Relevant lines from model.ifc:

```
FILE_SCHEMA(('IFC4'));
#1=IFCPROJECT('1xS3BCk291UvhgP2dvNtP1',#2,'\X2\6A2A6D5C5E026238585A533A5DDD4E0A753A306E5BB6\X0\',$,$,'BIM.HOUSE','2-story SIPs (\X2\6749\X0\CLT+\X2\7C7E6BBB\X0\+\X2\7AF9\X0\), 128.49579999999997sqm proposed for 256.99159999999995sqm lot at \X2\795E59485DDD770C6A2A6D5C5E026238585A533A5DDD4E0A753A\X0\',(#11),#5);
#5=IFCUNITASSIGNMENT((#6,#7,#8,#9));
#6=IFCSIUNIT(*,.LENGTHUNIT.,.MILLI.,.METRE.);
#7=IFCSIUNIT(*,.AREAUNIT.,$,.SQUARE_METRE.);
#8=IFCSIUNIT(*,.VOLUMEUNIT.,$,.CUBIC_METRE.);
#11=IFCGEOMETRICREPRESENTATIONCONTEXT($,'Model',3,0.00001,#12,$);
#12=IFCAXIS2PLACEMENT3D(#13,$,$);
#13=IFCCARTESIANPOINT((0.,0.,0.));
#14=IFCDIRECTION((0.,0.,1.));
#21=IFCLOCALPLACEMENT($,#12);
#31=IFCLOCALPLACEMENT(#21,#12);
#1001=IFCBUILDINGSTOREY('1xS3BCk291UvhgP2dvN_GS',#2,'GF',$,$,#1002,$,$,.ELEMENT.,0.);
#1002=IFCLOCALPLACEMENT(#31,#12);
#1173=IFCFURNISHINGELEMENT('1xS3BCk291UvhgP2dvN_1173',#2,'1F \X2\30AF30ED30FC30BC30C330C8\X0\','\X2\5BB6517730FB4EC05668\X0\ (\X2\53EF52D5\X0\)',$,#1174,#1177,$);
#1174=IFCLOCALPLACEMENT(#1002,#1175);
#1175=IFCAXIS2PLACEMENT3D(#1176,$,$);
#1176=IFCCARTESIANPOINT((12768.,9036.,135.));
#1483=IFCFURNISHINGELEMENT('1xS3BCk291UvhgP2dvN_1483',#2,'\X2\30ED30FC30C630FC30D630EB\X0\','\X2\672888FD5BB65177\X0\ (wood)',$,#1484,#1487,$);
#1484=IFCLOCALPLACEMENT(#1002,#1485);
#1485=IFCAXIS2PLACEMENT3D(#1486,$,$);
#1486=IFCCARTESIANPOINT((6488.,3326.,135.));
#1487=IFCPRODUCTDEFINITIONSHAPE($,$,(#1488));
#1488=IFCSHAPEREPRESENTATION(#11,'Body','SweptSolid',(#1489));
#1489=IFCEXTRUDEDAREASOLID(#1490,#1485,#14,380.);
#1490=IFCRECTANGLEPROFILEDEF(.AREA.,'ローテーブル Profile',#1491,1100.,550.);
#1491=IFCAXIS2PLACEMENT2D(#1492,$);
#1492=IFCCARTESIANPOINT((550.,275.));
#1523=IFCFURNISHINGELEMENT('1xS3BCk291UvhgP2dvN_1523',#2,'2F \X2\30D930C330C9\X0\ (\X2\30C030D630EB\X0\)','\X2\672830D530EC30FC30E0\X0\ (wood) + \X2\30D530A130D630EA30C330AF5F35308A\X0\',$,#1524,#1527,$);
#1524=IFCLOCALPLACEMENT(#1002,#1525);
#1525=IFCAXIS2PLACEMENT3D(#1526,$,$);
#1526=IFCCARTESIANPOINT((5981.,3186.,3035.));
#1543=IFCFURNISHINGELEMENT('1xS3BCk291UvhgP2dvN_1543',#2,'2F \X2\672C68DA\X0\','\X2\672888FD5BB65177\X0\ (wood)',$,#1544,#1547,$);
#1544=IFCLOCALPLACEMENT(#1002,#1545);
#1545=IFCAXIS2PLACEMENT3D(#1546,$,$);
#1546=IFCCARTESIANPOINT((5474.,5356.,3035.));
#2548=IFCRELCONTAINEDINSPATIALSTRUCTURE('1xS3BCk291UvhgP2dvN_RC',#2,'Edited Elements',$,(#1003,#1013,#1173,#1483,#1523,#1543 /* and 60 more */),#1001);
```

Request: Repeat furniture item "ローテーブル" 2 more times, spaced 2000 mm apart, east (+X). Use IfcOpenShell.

```python
import numpy as np
import ifcopenshell
import ifcopenshell.api.geometry
import ifcopenshell.api.root
import ifcopenshell.util.element
import ifcopenshell.util.placement
import ifcopenshell.util.unit

model = ifcopenshell.open("model.ifc")
unit_scale = ifcopenshell.util.unit.calculate_unit_scale(model)


def reuse_history(source, copy):
    """copy_class also copies each property set's owner history, people and application; keep the originals."""
    for rel in copy.IsDefinedBy:
        if rel.is_a("IfcRelDefinesByProperties") and (history := rel.RelatingPropertyDefinition.OwnerHistory):
            rel.RelatingPropertyDefinition.OwnerHistory = source.OwnerHistory
            ifcopenshell.util.element.remove_deep2(model, history)


source = model.by_guid("1xS3BCk291UvhgP2dvN_1483")
base = ifcopenshell.util.placement.get_local_placement(source.ObjectPlacement)
step = np.array([1.0, 0.0, 0.0]) * 2 / unit_scale

for i in range(1, 3):
    copy = ifcopenshell.api.root.copy_class(model, product=source)
    copy.Representation = ifcopenshell.util.element.copy_deep(
        model, source.Representation, exclude=["IfcGeometricRepresentationContext", "IfcRepresentationMap"]
    )
    reuse_history(source, copy)
    matrix = base.copy()
    matrix[:3, 3] += i * step
    print("added at", matrix[:3, 3].round(3) + 0.0)
    ifcopenshell.api.geometry.edit_object_placement(model, product=copy, matrix=matrix, is_si=False)

model.write("model_v2.ifc")
```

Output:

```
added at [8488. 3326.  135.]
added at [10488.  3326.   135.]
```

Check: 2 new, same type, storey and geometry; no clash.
